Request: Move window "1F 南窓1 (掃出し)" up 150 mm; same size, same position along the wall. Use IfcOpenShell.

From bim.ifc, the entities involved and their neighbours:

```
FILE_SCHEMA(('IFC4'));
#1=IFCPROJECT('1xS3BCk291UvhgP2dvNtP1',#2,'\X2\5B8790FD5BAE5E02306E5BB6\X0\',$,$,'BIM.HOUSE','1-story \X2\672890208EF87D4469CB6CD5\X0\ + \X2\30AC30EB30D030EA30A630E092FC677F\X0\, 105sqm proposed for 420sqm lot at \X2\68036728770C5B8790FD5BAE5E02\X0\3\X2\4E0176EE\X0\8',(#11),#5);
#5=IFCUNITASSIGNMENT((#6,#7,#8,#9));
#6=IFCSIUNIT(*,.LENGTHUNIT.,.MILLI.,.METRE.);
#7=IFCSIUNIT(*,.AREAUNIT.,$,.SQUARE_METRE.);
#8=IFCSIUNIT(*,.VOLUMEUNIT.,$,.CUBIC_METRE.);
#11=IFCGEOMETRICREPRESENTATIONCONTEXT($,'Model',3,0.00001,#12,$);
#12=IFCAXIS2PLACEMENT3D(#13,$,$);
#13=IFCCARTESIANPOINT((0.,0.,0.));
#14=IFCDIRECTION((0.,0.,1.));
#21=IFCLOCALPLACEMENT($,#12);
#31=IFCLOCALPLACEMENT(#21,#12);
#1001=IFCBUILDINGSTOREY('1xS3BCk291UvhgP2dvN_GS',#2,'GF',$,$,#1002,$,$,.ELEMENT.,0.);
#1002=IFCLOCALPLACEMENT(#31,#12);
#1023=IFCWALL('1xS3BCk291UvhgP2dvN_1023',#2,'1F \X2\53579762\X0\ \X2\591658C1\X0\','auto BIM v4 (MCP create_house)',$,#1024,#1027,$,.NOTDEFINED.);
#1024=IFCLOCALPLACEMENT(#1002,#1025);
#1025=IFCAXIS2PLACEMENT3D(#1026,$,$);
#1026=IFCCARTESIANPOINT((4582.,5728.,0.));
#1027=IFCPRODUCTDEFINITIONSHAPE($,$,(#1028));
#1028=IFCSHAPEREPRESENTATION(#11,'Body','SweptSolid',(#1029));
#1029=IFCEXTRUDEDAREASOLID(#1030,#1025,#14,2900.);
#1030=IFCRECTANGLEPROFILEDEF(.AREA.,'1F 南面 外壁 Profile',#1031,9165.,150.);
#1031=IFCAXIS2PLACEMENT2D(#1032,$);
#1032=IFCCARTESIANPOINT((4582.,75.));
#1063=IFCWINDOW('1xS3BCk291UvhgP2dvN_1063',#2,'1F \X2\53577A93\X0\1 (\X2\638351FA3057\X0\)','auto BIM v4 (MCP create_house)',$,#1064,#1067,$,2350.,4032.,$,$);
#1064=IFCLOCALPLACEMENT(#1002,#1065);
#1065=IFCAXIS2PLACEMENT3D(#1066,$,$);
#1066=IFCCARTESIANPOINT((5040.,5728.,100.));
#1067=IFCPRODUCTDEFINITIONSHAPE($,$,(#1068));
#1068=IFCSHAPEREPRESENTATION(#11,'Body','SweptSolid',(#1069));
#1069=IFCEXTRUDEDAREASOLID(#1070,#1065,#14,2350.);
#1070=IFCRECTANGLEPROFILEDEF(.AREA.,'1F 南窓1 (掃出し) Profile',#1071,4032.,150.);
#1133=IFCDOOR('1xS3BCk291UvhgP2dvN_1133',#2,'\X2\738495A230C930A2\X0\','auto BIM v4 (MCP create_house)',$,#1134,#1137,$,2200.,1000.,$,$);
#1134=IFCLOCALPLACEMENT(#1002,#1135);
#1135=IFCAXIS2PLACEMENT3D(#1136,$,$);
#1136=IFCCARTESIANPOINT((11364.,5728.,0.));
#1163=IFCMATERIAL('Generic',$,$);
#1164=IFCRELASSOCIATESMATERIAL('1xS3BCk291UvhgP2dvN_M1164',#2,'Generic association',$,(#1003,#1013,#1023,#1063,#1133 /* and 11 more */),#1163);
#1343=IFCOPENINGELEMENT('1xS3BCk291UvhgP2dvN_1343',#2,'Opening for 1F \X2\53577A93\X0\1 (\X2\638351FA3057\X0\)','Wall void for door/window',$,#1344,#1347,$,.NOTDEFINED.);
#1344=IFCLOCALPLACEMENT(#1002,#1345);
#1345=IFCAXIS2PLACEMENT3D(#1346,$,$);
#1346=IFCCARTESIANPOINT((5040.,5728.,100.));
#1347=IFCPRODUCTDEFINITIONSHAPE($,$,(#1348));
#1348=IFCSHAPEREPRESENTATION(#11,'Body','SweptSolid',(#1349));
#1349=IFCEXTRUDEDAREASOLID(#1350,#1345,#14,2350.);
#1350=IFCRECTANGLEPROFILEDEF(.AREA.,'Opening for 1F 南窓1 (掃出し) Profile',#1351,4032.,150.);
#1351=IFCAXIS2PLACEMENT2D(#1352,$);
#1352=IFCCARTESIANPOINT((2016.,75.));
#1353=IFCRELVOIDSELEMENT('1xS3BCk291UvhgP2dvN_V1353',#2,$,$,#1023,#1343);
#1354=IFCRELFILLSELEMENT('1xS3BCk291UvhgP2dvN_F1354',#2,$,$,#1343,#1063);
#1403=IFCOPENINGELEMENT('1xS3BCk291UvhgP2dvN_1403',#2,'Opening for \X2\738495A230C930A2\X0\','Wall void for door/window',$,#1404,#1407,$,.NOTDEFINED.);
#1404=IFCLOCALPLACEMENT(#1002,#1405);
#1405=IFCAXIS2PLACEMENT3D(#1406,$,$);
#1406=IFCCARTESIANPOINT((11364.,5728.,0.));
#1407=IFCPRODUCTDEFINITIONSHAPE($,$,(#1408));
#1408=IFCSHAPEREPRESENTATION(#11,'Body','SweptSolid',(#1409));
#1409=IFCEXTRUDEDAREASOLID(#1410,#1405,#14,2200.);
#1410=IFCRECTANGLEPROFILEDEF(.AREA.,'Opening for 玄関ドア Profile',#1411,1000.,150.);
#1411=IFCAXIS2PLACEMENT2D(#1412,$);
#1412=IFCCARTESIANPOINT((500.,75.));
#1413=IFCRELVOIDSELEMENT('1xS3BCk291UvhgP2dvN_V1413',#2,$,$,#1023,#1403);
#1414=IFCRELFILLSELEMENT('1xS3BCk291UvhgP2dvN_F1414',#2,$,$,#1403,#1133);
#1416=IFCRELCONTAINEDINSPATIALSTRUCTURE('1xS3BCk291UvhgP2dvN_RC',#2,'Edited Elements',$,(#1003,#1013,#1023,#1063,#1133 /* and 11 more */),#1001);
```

```python
import numpy as np
import ifcopenshell
import ifcopenshell.api.geometry
import ifcopenshell.util.placement
import ifcopenshell.util.unit

model = ifcopenshell.open("bim.ifc")
unit_scale = ifcopenshell.util.unit.calculate_unit_scale(model)

window = model.by_id(1063)
opening = window.FillsVoids[0].RelatingOpeningElement
dz = 150.0

shift = np.array([0.0, 0.0, dz])
# The window is not placed relative to its opening, so move both.
for product in (opening, window):
    matrix = ifcopenshell.util.placement.get_local_placement(product.ObjectPlacement)
    matrix[:3, 3] += shift
    ifcopenshell.api.geometry.edit_object_placement(model, product=product, matrix=matrix, is_si=False)

print(f"moved by {dz * unit_scale:+.3f} m")

model.write("bim_edited.ifc")
```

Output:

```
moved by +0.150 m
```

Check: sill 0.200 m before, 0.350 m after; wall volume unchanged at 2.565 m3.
